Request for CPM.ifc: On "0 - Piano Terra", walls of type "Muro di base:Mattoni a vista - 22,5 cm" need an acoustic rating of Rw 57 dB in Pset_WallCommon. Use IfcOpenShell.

First a look at what the model holds.

```python
import ifcopenshell
import ifcopenshell.util.element

model = ifcopenshell.open("CPM.ifc")
print(model.schema)
storey = next(s for s in model.by_type("IfcBuildingStorey") if s.Name == "0 - Piano Terra")
walls = [e for e in ifcopenshell.util.element.get_decomposition(storey) if e.is_a("IfcWall")]
seen = {}
for e in walls:
    element_type = ifcopenshell.util.element.get_type(e)
    key = (element_type.Name if element_type != e and element_type else None, ifcopenshell.util.element.get_pset(e, "Pset_WallCommon", "AcousticRating"))
    seen[key] = seen.get(key, 0) + 1
for (name, value), count in sorted(seen.items(), key=str):
    print(count, "x", name, "|", value)
```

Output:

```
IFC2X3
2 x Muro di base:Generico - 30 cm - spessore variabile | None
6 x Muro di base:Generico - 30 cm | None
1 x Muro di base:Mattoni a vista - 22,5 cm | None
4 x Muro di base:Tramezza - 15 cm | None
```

```python
import ifcopenshell
import ifcopenshell.api.pset
import ifcopenshell.util.element

model = ifcopenshell.open("CPM.ifc")

storey = next(s for s in model.by_type("IfcBuildingStorey") if s.Name == "0 - Piano Terra")
walls = [e for e in ifcopenshell.util.element.get_decomposition(storey) if e.is_a("IfcWall")]

count = 0
for e in walls:
    element_type = ifcopenshell.util.element.get_type(e)
    if element_type in (None, e) or element_type.Name != "Muro di base:Mattoni a vista - 22,5 cm":
        continue
    # add_pset returns the element's existing set when there is one.
    pset = ifcopenshell.api.pset.add_pset(model, product=e, name="Pset_WallCommon")
    ifcopenshell.api.pset.edit_pset(model, pset=pset, properties={"AcousticRating": "Rw 57 dB"})
    count += 1

print(count, "walls updated")

model.write("CPM-out.ifc")
```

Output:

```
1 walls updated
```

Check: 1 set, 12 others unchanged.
